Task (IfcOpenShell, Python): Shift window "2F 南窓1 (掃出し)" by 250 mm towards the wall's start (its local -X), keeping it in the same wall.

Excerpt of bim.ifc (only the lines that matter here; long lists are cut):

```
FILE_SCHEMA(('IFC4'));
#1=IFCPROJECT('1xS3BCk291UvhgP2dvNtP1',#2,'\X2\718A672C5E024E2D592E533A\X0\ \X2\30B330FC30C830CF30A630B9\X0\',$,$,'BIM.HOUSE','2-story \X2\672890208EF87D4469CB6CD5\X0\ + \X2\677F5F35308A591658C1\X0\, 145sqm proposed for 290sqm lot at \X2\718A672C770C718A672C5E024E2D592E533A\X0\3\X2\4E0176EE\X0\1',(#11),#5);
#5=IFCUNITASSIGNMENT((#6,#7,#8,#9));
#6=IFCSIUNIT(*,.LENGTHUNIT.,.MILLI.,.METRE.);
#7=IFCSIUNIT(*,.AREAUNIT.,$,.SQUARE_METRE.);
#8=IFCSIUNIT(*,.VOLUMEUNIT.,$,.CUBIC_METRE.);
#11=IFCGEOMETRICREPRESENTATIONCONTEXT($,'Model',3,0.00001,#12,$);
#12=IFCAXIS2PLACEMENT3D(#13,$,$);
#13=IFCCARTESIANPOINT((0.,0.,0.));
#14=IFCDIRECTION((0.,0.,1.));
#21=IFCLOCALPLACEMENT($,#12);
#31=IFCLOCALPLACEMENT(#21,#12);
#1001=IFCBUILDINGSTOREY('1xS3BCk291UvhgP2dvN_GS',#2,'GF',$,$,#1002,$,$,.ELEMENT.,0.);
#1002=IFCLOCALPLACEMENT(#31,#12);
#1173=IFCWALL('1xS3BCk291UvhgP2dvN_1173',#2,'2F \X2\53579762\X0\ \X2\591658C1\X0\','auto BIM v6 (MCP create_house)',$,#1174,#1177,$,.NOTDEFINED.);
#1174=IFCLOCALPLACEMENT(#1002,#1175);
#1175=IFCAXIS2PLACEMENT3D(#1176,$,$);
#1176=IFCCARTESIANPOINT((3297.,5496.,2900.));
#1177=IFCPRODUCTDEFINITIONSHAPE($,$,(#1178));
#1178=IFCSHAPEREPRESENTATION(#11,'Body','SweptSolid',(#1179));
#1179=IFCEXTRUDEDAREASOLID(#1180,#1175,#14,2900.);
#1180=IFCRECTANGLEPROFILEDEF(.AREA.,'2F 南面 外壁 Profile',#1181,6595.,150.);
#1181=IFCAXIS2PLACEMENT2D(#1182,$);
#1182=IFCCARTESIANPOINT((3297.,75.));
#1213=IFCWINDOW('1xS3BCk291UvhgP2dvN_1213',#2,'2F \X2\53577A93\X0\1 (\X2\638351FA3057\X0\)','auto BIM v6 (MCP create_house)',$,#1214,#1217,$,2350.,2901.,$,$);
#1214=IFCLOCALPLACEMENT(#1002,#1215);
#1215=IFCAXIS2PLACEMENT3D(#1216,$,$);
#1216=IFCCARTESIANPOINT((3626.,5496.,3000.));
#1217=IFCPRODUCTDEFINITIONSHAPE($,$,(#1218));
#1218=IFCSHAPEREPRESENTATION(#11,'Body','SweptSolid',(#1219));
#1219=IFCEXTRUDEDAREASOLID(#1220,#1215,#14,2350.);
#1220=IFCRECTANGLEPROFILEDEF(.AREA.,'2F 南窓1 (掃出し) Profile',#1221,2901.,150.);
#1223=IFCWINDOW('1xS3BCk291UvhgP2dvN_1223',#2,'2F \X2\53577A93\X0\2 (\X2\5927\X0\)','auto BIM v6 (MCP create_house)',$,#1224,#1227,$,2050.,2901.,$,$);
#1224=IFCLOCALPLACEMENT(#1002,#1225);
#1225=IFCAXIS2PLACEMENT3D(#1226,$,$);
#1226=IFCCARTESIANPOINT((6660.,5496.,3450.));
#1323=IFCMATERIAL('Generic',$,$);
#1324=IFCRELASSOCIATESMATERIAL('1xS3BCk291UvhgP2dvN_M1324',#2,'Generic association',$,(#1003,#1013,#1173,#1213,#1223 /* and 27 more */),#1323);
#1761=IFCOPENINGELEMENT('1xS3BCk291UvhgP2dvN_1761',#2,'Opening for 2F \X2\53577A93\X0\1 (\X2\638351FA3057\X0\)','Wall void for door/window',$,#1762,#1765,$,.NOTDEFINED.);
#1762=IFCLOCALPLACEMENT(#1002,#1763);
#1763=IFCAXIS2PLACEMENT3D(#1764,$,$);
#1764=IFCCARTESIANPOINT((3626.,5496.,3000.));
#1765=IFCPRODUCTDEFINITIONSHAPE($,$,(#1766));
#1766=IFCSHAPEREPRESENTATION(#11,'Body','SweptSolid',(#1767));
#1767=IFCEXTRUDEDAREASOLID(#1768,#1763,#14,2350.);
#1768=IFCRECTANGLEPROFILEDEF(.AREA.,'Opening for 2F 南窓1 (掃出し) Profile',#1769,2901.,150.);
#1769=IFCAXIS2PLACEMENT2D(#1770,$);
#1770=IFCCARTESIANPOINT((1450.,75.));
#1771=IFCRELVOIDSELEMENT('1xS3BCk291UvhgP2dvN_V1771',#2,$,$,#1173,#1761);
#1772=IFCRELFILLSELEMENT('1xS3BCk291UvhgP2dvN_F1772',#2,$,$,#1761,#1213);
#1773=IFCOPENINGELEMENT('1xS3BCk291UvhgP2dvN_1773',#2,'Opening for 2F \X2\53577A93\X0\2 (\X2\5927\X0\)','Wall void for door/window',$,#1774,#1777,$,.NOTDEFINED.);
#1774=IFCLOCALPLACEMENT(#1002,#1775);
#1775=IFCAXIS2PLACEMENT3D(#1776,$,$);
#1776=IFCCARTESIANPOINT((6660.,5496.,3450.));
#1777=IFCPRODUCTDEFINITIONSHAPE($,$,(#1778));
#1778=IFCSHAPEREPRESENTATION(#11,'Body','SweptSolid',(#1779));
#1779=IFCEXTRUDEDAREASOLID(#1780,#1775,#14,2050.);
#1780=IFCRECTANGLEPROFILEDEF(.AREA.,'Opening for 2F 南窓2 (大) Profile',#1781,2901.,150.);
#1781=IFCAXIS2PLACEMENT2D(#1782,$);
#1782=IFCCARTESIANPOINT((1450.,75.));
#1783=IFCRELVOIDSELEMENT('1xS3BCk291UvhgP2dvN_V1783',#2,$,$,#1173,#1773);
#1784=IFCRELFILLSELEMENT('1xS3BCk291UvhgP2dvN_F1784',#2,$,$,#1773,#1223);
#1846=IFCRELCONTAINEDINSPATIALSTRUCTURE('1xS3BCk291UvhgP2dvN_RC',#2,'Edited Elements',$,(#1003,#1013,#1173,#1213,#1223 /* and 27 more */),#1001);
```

```python
import ifcopenshell
import ifcopenshell.api.geometry
import ifcopenshell.util.placement

model = ifcopenshell.open("bim.ifc")

window = model.by_guid("1xS3BCk291UvhgP2dvN_1213")
opening = window.FillsVoids[0].RelatingOpeningElement
wall = opening.VoidsElements[0].RelatingBuildingElement

wall_matrix = ifcopenshell.util.placement.get_local_placement(wall.ObjectPlacement)
shift = wall_matrix[:3, 0] * -250.0
before = ifcopenshell.util.placement.get_local_placement(window.ObjectPlacement)[:3, 3].copy()

# The window is not placed relative to its opening, so move both.
for product in (opening, window):
    matrix = ifcopenshell.util.placement.get_local_placement(product.ObjectPlacement)
    matrix[:3, 3] += shift
    ifcopenshell.api.geometry.edit_object_placement(model, product=product, matrix=matrix, is_si=False)

after = ifcopenshell.util.placement.get_local_placement(window.ObjectPlacement)[:3, 3]
print("window moved by", (after - before).round(3) + 0.0)

model.write("bim-out.ifc")
```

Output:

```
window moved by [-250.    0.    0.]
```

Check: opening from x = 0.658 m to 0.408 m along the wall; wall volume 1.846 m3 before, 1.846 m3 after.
